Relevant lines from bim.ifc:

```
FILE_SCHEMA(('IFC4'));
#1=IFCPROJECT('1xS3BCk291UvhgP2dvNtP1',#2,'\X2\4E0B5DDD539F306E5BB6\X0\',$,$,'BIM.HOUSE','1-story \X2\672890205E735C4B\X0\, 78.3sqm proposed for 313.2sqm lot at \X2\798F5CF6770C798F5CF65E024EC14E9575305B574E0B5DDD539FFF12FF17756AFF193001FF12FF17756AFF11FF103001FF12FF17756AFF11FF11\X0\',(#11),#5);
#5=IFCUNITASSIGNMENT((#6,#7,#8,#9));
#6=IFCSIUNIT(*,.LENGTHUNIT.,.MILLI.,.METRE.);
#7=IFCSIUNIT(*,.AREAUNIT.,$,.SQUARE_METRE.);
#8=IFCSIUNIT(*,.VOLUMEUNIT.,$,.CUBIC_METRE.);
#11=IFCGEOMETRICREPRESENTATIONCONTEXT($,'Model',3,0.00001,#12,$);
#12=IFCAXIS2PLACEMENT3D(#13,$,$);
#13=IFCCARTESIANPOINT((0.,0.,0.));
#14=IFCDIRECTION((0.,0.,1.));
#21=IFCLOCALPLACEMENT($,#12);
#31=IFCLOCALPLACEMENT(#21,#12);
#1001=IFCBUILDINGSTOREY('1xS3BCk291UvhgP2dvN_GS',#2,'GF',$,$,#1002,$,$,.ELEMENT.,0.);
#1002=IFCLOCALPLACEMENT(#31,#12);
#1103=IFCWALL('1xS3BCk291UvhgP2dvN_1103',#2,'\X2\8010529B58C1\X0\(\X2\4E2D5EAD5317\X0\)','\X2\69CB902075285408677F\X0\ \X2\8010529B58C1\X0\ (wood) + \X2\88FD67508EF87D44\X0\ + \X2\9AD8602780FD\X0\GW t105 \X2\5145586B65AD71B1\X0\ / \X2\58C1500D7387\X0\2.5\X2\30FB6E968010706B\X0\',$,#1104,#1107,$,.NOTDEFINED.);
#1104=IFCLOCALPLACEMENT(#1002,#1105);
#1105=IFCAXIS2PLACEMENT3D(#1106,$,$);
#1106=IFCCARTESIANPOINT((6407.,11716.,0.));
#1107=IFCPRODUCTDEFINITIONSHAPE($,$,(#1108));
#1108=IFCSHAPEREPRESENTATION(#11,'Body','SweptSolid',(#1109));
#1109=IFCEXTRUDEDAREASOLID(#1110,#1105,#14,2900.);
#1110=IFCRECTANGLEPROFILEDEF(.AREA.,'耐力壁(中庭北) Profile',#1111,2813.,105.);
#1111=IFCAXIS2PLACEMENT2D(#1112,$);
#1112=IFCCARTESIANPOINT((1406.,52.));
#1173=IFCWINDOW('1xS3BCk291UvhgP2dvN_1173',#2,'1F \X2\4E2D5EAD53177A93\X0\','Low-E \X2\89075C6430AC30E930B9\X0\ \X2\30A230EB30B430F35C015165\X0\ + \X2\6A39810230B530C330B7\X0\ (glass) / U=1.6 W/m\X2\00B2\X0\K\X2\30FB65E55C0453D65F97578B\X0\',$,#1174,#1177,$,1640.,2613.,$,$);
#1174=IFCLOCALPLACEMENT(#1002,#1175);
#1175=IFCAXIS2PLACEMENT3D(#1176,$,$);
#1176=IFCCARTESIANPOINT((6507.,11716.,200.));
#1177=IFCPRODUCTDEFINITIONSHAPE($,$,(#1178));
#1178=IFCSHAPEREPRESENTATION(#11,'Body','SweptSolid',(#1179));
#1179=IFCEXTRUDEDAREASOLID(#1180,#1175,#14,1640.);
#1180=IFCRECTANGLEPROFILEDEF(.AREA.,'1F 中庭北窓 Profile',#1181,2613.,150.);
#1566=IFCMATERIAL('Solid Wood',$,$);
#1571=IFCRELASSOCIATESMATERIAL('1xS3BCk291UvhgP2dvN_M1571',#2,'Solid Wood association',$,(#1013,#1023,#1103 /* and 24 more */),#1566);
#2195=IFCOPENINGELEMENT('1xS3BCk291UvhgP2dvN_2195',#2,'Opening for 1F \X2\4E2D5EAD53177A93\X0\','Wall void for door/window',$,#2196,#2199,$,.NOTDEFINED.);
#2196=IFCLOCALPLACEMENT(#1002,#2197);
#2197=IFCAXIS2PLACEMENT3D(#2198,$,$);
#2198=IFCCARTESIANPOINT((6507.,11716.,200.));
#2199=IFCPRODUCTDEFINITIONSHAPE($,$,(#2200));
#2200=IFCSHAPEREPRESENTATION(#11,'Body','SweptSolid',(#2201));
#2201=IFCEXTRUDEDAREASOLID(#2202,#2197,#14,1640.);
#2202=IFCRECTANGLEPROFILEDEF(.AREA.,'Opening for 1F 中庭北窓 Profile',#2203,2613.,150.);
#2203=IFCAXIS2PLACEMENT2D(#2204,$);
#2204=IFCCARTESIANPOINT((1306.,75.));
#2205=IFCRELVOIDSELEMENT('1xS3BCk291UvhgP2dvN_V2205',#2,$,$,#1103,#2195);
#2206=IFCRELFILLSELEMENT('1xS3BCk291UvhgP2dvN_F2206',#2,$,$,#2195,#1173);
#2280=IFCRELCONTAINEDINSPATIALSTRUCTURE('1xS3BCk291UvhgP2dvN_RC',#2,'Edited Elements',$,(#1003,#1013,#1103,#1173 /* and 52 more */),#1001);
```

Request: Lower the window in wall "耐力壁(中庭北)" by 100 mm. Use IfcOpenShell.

```python
import numpy as np
import ifcopenshell
import ifcopenshell.api.geometry
import ifcopenshell.util.placement
import ifcopenshell.util.unit

model = ifcopenshell.open("bim.ifc")
unit_scale = ifcopenshell.util.unit.calculate_unit_scale(model)

window = model.by_guid("1xS3BCk291UvhgP2dvN_1173")
opening = window.FillsVoids[0].RelatingOpeningElement
dz = -0.1 / unit_scale

shift = np.array([0.0, 0.0, dz])
# The window is not placed relative to its opening, so move both.
for product in (opening, window):
    matrix = ifcopenshell.util.placement.get_local_placement(product.ObjectPlacement)
    matrix[:3, 3] += shift
    ifcopenshell.api.geometry.edit_object_placement(model, product=product, matrix=matrix, is_si=False)

print(f"moved by {dz * unit_scale:+.3f} m")

model.write("bim_rev.ifc")
```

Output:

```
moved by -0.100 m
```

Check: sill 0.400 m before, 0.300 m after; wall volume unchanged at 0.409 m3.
